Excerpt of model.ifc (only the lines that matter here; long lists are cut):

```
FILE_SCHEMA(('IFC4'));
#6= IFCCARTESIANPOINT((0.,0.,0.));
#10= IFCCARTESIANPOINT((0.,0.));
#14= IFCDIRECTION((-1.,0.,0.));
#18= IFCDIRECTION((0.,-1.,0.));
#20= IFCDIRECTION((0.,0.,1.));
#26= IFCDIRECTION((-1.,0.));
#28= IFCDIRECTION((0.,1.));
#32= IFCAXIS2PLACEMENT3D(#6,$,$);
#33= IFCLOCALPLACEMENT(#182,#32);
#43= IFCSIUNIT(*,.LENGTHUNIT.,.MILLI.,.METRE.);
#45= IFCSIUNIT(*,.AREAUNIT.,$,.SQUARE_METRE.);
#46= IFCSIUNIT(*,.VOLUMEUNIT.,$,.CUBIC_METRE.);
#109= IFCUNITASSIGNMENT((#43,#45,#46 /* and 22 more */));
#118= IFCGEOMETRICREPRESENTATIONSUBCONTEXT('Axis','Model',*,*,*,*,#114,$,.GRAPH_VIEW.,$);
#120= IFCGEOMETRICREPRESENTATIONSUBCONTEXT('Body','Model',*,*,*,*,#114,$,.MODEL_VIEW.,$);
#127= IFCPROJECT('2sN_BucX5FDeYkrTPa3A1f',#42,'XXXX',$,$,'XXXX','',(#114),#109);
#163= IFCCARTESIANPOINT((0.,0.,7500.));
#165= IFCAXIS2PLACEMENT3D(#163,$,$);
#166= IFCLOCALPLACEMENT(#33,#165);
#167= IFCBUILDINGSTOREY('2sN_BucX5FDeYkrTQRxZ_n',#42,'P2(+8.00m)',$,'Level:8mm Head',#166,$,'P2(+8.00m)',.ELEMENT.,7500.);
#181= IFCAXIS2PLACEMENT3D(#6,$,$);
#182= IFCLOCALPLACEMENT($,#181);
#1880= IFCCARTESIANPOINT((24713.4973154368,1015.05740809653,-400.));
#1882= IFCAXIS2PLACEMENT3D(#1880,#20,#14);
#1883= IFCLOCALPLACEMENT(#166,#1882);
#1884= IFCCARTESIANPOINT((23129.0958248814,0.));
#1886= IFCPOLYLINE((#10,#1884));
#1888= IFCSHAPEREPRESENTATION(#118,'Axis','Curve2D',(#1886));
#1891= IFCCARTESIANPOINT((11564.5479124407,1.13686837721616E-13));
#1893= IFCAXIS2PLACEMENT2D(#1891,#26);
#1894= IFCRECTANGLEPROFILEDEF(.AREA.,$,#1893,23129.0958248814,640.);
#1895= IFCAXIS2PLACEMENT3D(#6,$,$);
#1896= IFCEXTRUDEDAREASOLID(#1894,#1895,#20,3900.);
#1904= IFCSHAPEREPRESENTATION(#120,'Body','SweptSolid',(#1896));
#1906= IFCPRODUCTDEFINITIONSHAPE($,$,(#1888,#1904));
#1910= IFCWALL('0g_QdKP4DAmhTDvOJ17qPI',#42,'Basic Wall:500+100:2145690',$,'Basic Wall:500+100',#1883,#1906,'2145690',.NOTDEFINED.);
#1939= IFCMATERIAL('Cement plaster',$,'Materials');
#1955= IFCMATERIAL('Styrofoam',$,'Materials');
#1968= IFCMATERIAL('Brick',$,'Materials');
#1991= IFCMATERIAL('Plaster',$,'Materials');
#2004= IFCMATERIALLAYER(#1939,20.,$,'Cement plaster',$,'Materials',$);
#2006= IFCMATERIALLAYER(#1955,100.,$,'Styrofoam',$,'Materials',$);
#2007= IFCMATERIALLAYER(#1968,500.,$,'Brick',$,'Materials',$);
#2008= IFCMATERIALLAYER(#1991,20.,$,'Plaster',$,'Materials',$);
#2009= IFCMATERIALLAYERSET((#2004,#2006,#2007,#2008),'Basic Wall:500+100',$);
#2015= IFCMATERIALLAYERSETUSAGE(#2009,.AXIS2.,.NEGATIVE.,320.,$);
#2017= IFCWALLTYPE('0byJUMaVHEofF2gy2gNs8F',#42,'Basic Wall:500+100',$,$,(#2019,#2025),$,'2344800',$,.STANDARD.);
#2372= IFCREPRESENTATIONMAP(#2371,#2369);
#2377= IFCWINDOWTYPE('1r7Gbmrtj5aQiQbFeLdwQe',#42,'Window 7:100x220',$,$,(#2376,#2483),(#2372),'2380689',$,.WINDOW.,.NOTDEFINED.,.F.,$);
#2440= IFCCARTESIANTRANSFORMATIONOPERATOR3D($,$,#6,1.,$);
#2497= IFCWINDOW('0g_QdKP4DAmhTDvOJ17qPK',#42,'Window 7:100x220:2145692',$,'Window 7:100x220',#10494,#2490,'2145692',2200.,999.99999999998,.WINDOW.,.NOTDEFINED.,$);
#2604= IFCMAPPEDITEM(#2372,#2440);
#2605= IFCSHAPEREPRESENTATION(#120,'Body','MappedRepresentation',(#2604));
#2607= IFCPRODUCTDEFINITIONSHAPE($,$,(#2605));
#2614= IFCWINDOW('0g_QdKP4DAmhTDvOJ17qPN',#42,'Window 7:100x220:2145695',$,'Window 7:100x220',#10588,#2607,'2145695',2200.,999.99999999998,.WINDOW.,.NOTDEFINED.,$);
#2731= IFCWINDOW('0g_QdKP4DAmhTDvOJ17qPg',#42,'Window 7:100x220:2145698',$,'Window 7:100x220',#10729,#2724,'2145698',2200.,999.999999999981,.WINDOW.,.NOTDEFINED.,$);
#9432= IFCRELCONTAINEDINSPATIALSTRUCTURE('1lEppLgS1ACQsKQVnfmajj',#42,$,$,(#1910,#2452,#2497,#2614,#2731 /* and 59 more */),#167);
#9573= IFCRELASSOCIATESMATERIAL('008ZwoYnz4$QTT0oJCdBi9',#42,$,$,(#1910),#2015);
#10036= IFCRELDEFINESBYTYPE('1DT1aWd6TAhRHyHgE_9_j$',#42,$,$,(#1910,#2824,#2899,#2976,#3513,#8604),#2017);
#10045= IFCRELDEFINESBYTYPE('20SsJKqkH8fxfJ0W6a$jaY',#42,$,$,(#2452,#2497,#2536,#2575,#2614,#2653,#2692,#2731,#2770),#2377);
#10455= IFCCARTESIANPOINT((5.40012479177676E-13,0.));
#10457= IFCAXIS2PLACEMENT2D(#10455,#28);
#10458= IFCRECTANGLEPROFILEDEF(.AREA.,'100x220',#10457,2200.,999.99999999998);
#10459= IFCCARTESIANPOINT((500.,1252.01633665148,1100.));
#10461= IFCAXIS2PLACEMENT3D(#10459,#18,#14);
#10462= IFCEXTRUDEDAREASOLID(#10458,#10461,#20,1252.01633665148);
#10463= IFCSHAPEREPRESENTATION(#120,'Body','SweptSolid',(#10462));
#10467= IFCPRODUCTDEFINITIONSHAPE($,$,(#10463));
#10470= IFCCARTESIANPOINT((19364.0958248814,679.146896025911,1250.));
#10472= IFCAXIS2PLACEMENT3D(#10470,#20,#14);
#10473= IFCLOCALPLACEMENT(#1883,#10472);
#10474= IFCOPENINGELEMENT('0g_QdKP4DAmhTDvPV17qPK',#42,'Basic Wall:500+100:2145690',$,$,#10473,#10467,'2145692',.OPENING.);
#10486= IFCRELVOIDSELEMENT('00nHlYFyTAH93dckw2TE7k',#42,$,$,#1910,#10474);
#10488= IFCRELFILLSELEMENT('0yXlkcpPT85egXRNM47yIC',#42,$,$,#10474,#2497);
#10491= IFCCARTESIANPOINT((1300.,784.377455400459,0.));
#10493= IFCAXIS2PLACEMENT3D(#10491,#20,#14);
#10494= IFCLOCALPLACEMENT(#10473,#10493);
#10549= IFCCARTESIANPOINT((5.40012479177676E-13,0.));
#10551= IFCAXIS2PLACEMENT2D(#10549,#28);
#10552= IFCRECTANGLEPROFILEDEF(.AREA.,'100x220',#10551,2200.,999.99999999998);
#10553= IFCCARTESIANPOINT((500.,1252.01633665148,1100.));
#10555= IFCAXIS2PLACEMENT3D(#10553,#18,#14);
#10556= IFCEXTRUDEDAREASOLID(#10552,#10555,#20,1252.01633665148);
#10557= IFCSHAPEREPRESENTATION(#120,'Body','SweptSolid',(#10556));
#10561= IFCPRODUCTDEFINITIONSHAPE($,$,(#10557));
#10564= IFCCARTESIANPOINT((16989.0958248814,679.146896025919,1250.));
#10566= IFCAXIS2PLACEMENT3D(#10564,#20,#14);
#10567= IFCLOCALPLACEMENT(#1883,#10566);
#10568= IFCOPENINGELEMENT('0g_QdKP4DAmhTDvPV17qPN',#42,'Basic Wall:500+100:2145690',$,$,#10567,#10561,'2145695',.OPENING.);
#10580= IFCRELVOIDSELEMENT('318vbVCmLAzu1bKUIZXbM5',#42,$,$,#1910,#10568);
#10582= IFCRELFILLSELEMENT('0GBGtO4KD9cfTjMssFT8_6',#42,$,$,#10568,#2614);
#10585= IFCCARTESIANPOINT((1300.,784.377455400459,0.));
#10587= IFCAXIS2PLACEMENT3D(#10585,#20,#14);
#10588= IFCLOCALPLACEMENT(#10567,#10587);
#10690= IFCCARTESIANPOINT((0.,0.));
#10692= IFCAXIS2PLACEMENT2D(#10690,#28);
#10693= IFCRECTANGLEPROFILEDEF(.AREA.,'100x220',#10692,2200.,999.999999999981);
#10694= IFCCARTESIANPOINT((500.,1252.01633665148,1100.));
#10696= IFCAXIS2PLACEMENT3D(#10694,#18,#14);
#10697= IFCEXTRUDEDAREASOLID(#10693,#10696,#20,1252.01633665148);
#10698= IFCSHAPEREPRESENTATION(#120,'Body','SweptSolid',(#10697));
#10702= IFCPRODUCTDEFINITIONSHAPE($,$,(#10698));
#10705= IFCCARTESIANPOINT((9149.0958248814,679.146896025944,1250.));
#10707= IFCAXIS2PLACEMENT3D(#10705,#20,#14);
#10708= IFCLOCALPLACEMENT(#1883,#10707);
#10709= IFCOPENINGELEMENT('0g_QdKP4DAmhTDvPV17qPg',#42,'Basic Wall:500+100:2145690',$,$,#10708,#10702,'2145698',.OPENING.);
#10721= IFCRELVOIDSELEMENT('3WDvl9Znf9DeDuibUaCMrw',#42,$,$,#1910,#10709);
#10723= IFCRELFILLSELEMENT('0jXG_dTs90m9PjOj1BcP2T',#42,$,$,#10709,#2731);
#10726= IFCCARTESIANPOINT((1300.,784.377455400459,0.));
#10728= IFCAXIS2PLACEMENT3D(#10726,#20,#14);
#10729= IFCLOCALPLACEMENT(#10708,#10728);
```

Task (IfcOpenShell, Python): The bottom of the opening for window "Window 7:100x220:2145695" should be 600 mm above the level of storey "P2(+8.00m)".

```python
import numpy as np
import ifcopenshell
import ifcopenshell.api.geometry
import ifcopenshell.geom
import ifcopenshell.util.element
import ifcopenshell.util.placement
import ifcopenshell.util.shape
import ifcopenshell.util.unit

model = ifcopenshell.open("model.ifc")
unit_scale = ifcopenshell.util.unit.calculate_unit_scale(model)

window = model.by_guid("0g_QdKP4DAmhTDvOJ17qPN")
opening = window.FillsVoids[0].RelatingOpeningElement
storey = ifcopenshell.util.element.get_container(window, ifc_class="IfcBuildingStorey")
level = ifcopenshell.util.placement.get_local_placement(storey.ObjectPlacement)[2, 3]

# The opening's origin need not be at the sill, so measure its lowest point.
shape = ifcopenshell.geom.create_shape(ifcopenshell.geom.settings(), opening)
bottom = ifcopenshell.util.shape.get_shape_bottom_elevation(shape, shape.geometry) / unit_scale
dz = level + 0.6 / unit_scale - bottom

shift = np.array([0.0, 0.0, dz])
# The window is placed relative to its opening, so it follows when the opening moves.
matrix = ifcopenshell.util.placement.get_local_placement(opening.ObjectPlacement)
matrix[:3, 3] += shift
ifcopenshell.api.geometry.edit_object_placement(
    model, product=opening, matrix=matrix, is_si=False, should_transform_children=True
)

print(f"moved by {dz * unit_scale:+.3f} m")

model.write("model-out.ifc")
```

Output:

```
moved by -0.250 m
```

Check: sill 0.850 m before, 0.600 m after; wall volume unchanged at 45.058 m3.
